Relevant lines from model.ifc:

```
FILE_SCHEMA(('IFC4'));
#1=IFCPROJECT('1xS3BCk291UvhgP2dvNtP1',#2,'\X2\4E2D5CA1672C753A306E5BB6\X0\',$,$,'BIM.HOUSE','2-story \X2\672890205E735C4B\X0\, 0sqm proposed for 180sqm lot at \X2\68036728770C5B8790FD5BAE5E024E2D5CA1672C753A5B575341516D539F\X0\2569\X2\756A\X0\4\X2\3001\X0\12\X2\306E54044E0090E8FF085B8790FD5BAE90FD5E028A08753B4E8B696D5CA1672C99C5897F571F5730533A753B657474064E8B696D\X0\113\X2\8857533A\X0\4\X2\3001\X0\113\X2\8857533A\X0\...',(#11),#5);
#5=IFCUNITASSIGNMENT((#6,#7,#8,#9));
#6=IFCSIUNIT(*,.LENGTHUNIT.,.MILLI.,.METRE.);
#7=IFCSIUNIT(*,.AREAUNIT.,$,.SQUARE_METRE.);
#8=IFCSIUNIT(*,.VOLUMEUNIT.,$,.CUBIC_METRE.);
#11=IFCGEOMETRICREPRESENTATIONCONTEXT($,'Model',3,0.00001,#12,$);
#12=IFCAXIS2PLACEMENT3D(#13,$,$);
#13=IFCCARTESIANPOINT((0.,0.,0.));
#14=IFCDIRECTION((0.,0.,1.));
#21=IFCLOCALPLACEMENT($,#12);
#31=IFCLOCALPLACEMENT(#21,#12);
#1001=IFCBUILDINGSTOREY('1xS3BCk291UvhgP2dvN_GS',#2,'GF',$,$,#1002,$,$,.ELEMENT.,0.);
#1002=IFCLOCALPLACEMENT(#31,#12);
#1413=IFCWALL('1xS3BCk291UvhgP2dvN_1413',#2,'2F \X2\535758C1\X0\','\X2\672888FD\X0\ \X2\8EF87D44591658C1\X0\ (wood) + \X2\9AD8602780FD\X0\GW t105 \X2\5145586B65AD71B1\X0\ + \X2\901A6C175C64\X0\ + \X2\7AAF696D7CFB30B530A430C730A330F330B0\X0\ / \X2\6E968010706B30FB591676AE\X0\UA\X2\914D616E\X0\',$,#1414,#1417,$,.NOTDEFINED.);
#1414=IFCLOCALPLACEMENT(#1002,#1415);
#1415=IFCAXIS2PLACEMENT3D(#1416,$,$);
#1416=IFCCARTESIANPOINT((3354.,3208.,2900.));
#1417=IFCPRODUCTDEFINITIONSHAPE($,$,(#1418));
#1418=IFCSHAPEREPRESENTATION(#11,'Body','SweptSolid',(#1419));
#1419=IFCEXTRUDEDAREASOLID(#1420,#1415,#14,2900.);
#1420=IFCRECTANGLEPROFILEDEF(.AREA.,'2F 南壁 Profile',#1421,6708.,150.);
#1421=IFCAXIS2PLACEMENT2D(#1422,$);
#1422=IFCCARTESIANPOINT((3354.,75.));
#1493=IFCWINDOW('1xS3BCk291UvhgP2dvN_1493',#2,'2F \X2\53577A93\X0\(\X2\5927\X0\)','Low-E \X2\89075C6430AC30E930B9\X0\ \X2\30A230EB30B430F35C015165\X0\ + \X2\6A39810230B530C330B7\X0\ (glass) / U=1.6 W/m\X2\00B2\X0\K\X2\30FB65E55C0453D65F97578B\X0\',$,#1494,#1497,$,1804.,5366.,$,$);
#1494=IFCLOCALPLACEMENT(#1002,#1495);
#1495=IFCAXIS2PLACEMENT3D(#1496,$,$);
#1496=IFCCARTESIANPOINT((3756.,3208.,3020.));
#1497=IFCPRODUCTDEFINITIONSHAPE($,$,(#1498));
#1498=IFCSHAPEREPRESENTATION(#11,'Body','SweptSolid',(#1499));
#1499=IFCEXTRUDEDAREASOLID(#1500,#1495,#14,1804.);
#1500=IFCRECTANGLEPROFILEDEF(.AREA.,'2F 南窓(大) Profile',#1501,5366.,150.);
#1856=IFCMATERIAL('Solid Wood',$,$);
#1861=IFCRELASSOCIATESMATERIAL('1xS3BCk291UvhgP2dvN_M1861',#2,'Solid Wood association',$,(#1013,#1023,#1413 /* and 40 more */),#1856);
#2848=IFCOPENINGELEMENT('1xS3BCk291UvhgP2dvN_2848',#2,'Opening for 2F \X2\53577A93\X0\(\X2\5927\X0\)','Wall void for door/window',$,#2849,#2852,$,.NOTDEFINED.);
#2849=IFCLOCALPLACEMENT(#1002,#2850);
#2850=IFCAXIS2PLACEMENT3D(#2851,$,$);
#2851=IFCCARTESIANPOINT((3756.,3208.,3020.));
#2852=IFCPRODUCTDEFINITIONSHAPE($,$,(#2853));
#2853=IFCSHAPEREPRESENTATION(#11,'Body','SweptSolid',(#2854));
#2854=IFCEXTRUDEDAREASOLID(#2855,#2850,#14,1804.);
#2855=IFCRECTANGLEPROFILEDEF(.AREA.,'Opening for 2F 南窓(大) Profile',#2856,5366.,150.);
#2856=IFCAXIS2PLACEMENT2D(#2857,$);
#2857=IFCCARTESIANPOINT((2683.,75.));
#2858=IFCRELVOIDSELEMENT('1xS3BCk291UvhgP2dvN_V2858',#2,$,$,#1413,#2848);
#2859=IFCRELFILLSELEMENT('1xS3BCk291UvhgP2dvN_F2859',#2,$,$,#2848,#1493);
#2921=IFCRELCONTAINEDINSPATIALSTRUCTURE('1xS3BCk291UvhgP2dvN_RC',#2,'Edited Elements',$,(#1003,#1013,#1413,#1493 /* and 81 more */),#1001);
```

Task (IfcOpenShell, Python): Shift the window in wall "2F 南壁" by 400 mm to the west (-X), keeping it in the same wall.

```python
import ifcopenshell
import ifcopenshell.api.geometry
import ifcopenshell.util.placement

model = ifcopenshell.open("model.ifc")

window = model.by_guid("1xS3BCk291UvhgP2dvN_1493")
opening = window.FillsVoids[0].RelatingOpeningElement
wall = opening.VoidsElements[0].RelatingBuildingElement

wall_matrix = ifcopenshell.util.placement.get_local_placement(wall.ObjectPlacement)
shift = wall_matrix[:3, 0] * -400.0
before = ifcopenshell.util.placement.get_local_placement(window.ObjectPlacement)[:3, 3].copy()

# The window is not placed relative to its opening, so move both.
for product in (opening, window):
    matrix = ifcopenshell.util.placement.get_local_placement(product.ObjectPlacement)
    matrix[:3, 3] += shift
    ifcopenshell.api.geometry.edit_object_placement(model, product=product, matrix=matrix, is_si=False)

after = ifcopenshell.util.placement.get_local_placement(window.ObjectPlacement)[:3, 3]
print("window moved by", (after - before).round(3) + 0.0)

model.write("model_updated.ifc")
```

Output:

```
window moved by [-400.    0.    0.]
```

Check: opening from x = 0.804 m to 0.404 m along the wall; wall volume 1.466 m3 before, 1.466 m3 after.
